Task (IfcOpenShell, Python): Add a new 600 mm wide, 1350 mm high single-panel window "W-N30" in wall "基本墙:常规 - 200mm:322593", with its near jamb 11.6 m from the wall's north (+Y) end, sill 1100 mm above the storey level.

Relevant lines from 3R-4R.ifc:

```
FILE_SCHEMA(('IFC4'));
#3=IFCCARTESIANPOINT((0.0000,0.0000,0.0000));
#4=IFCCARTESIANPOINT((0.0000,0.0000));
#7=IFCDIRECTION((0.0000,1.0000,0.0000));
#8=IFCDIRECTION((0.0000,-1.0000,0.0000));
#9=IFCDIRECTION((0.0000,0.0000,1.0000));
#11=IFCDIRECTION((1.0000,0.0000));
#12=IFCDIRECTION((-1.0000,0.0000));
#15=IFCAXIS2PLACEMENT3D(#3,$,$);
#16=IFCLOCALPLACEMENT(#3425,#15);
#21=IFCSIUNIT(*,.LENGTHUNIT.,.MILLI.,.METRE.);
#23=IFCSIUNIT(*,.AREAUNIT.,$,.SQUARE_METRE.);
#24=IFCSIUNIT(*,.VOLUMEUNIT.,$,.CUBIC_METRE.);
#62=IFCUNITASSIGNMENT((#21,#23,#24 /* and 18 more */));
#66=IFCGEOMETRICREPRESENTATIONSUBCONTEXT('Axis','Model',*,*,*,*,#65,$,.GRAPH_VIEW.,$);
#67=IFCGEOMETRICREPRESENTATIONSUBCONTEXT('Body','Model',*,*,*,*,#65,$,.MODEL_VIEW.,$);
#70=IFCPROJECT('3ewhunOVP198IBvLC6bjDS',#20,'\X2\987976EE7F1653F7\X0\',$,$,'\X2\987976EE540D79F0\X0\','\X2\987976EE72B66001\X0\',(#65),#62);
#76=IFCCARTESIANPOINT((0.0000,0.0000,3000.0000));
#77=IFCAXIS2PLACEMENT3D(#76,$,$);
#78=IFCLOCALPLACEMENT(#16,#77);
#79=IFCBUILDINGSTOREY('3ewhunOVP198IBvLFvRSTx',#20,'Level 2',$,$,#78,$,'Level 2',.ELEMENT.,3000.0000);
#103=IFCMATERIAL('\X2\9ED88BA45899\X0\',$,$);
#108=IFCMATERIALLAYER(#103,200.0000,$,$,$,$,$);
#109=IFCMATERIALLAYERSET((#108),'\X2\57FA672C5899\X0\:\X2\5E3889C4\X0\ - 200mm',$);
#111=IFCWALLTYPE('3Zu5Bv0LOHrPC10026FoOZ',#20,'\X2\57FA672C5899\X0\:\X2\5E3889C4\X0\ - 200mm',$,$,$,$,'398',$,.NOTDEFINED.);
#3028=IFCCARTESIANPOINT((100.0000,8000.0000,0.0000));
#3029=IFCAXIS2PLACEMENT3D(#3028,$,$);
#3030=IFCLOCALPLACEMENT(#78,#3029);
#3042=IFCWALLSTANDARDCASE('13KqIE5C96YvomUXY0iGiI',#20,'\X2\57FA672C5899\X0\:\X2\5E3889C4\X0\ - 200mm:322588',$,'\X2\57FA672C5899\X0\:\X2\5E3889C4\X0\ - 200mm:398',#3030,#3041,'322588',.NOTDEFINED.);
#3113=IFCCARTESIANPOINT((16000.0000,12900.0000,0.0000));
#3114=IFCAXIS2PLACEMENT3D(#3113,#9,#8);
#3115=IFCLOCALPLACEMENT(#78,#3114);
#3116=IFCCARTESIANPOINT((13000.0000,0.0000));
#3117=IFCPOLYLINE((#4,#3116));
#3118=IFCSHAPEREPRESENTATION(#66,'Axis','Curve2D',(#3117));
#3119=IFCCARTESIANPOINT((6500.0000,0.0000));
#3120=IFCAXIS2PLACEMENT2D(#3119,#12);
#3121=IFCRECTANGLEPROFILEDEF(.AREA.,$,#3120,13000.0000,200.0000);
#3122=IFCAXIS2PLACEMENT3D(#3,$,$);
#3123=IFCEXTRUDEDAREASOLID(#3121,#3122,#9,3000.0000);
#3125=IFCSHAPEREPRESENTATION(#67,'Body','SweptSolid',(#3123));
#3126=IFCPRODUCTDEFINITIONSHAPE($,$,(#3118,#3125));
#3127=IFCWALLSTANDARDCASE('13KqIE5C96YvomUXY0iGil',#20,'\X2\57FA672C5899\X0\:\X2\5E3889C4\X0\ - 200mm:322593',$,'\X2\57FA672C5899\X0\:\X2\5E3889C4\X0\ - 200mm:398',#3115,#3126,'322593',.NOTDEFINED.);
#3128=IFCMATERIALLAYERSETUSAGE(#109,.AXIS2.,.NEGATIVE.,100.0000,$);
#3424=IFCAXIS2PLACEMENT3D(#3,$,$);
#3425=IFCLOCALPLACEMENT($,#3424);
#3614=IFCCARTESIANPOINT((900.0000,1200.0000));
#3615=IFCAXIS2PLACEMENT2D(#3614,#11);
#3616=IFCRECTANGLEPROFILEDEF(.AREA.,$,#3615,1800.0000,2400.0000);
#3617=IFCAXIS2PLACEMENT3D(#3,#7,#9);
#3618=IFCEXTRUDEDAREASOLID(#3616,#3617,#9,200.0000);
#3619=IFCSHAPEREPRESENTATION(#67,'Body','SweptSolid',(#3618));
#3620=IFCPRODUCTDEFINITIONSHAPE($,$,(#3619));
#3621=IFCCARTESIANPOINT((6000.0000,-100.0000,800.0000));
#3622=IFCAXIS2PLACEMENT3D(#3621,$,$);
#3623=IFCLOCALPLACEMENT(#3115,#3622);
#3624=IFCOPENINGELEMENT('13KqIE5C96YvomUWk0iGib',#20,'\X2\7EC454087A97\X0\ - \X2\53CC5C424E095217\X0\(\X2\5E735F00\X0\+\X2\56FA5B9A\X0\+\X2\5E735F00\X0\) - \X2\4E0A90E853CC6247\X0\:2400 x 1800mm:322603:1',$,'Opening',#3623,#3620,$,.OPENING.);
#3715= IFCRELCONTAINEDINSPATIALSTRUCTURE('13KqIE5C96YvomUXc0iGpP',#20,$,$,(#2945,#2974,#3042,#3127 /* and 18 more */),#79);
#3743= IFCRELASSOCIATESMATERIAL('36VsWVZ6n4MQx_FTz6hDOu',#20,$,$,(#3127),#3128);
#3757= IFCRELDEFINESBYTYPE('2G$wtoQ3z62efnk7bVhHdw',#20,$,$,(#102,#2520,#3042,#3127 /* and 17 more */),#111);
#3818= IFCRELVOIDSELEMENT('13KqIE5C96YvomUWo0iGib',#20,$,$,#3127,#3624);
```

```python
import numpy as np
import ifcopenshell
import ifcopenshell.api.feature
import ifcopenshell.api.geometry
import ifcopenshell.api.root
import ifcopenshell.api.spatial
import ifcopenshell.geom
import ifcopenshell.util.element
import ifcopenshell.util.placement
import ifcopenshell.util.representation
import ifcopenshell.util.shape
import ifcopenshell.util.unit

model = ifcopenshell.open("3R-4R.ifc")
unit_scale = ifcopenshell.util.unit.calculate_unit_scale(model)
settings = ifcopenshell.geom.settings()


def volume(element):
    """Net volume in cubic metres, openings subtracted."""
    shape = ifcopenshell.geom.create_shape(settings, element)
    return ifcopenshell.util.shape.get_volume(shape.geometry)


wall = model.by_id(3127)
storey = ifcopenshell.util.element.get_container(wall, ifc_class="IfcBuildingStorey")
context = ifcopenshell.util.representation.get_context(model, "Model", "Body", "MODEL_VIEW")
before = volume(wall)

width, height, from_end, sill = 0.6, 1.35, 11.6, 1.1  # metres

# The wall runs along its own X axis, and the end named is its -X end.
wall_shape = ifcopenshell.geom.create_shape(settings, wall)
x, y, z = ifcopenshell.util.shape.get_vertices(wall_shape.geometry).T
start = x.min() + from_end
face, thickness = float(y.min()), float(y.max() - y.min())
wall_matrix = ifcopenshell.util.placement.get_local_placement(wall.ObjectPlacement)
level = ifcopenshell.util.placement.get_local_placement(storey.ObjectPlacement)[2, 3]


def in_wall(x, y):
    """Placement at x, y metres in the wall's axes, at sill height."""
    matrix = wall_matrix.copy()
    matrix[:, 3] = wall_matrix @ np.array([x / unit_scale, y / unit_scale, 0.0, 1.0])
    matrix[2, 3] = level + sill / unit_scale
    return matrix


# Opening: a box that overshoots both wall faces by 50 mm.
opening = ifcopenshell.api.root.create_entity(model, ifc_class="IfcOpeningElement", predefined_type="OPENING")
box = ifcopenshell.api.geometry.add_wall_representation(
    model, context=context, length=width, height=height, thickness=thickness + 0.1
)
ifcopenshell.api.geometry.assign_representation(model, product=opening, representation=box)
ifcopenshell.api.geometry.edit_object_placement(model, product=opening, matrix=in_wall(start, face - 0.05), is_si=False)
ifcopenshell.api.feature.add_feature(model, feature=opening, element=wall)

window = ifcopenshell.api.root.create_entity(model, ifc_class="IfcWindow", name="W-N30", predefined_type="WINDOW")
window.OverallWidth, window.OverallHeight = width / unit_scale, height / unit_scale
window.PartitioningType = "SINGLE_PANEL"
body = ifcopenshell.api.geometry.add_window_representation(
    model,
    context=context,
    overall_width=window.OverallWidth,
    overall_height=window.OverallHeight,
    partition_type="SINGLE_PANEL",
)
ifcopenshell.api.geometry.assign_representation(model, product=window, representation=body)
ifcopenshell.api.spatial.assign_container(model, products=[window], relating_structure=storey)
ifcopenshell.api.feature.add_filling(model, opening=opening, element=window)

# Centre the window in the wall's thickness.
ifcopenshell.api.geometry.edit_object_placement(model, product=window, matrix=in_wall(start, face), is_si=False)
window_shape = ifcopenshell.geom.create_shape(settings, window)
depth = ifcopenshell.util.shape.get_vertices(window_shape.geometry)[:, 1]
offset = face + thickness / 2 - (depth.min() + depth.max()) / 2
ifcopenshell.api.geometry.edit_object_placement(model, product=window, matrix=in_wall(start, offset), is_si=False)

after = volume(wall)

print(f"wall volume {before:.3f} -> {after:.3f} m3")

model.write("3R-4R_v2.ifc")
```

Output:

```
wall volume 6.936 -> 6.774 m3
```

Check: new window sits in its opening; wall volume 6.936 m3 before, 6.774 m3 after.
